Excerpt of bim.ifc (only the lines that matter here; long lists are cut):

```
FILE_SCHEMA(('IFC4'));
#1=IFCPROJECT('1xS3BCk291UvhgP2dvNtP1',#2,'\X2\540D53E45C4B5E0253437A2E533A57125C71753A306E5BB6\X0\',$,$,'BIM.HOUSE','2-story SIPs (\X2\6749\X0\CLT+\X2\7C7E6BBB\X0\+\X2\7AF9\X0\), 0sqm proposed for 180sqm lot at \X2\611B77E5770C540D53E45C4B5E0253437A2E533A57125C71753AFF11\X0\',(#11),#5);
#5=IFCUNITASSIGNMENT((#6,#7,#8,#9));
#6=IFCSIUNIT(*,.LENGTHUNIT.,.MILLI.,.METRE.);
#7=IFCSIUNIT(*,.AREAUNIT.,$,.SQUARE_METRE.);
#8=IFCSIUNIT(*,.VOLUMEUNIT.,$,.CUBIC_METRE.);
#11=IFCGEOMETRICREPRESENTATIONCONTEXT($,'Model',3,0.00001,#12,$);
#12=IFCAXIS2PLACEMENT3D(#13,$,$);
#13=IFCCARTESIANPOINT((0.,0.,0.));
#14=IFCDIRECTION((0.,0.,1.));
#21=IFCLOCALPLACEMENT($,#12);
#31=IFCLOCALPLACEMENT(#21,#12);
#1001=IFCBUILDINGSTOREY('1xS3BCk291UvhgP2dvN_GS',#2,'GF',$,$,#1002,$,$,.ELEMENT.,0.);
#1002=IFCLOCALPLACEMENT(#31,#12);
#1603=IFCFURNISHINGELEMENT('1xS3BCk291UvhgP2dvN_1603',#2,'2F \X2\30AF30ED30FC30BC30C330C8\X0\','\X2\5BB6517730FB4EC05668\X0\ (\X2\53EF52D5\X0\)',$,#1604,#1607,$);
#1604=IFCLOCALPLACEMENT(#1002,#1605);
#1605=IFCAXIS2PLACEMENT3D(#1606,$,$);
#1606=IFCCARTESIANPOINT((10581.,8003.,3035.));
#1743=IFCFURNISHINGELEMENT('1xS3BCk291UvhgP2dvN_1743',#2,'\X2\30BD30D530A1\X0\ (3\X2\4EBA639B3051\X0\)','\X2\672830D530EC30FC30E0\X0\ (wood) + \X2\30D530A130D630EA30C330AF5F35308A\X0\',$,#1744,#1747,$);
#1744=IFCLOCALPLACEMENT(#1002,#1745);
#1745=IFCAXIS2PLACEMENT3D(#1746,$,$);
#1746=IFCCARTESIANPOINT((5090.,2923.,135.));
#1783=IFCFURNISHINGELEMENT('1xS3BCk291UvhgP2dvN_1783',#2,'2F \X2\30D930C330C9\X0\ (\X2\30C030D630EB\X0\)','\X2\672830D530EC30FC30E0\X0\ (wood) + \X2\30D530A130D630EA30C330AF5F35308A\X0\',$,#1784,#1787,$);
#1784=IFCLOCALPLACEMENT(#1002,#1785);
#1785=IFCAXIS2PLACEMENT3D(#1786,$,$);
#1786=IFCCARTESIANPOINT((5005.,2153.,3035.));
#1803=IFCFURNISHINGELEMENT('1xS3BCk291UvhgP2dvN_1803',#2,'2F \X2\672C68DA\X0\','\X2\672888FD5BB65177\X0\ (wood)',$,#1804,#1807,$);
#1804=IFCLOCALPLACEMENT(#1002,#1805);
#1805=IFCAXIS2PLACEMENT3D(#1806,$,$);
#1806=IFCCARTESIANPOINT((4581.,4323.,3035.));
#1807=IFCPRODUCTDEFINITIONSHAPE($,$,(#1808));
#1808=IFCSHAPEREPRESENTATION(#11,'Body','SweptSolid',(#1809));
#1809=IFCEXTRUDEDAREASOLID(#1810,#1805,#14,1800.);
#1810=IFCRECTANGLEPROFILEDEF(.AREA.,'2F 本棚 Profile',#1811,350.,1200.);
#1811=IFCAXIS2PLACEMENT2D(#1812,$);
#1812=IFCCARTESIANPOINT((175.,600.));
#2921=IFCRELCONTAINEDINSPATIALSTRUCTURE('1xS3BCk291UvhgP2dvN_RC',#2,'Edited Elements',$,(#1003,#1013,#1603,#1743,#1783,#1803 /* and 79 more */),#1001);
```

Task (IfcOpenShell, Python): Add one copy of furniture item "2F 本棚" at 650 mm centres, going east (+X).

```python
import numpy as np
import ifcopenshell
import ifcopenshell.api.geometry
import ifcopenshell.api.root
import ifcopenshell.util.element
import ifcopenshell.util.placement
import ifcopenshell.util.unit

model = ifcopenshell.open("bim.ifc")
unit_scale = ifcopenshell.util.unit.calculate_unit_scale(model)


def reuse_history(source, copy):
    """copy_class also copies each property set's owner history, people and application; keep the originals."""
    for rel in copy.IsDefinedBy:
        if rel.is_a("IfcRelDefinesByProperties") and (history := rel.RelatingPropertyDefinition.OwnerHistory):
            rel.RelatingPropertyDefinition.OwnerHistory = source.OwnerHistory
            ifcopenshell.util.element.remove_deep2(model, history)


source = model.by_id(1803)
base = ifcopenshell.util.placement.get_local_placement(source.ObjectPlacement)
step = np.array([1.0, 0.0, 0.0]) * 0.65 / unit_scale

for i in range(1, 2):
    copy = ifcopenshell.api.root.copy_class(model, product=source)
    copy.Representation = ifcopenshell.util.element.copy_deep(
        model, source.Representation, exclude=["IfcGeometricRepresentationContext", "IfcRepresentationMap"]
    )
    reuse_history(source, copy)
    matrix = base.copy()
    matrix[:3, 3] += i * step
    print("added at", matrix[:3, 3].round(3) + 0.0)
    ifcopenshell.api.geometry.edit_object_placement(model, product=copy, matrix=matrix, is_si=False)

model.write("bim_v2.ifc")
```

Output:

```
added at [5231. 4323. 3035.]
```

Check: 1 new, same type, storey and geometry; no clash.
